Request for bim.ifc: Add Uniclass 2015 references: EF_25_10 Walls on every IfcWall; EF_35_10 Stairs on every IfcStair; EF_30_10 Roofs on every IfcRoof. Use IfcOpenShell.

First a look at what the model holds.

```python
import ifcopenshell

model = ifcopenshell.open("bim.ifc")
print(model.schema)
print("classifications:", [c.Name for c in model.by_type("IfcClassification")])
for ifc_class in ("IfcDoor", "IfcRoof", "IfcStair", "IfcWall", "IfcWindow"):
    print(ifc_class, len(model.by_type(ifc_class)))
```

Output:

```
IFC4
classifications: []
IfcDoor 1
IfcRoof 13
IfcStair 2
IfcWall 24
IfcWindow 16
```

```python
import ifcopenshell
import ifcopenshell.api.classification

model = ifcopenshell.open("bim.ifc")

system = ifcopenshell.api.classification.add_classification(model, classification="Uniclass 2015")

codes = {
    "IfcWall": ("EF_25_10", "Walls"),
    "IfcStair": ("EF_35_10", "Stairs"),
    "IfcRoof": ("EF_30_10", "Roofs"),
}
for ifc_class, (code, name) in codes.items():
    products = model.by_type(ifc_class)
    ifcopenshell.api.classification.add_reference(
        model, products=products, classification=system, identification=code, name=name
    )
    print(code, len(products))

model.write("bim_rev.ifc")
```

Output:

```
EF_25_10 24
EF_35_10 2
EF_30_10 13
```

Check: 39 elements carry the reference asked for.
